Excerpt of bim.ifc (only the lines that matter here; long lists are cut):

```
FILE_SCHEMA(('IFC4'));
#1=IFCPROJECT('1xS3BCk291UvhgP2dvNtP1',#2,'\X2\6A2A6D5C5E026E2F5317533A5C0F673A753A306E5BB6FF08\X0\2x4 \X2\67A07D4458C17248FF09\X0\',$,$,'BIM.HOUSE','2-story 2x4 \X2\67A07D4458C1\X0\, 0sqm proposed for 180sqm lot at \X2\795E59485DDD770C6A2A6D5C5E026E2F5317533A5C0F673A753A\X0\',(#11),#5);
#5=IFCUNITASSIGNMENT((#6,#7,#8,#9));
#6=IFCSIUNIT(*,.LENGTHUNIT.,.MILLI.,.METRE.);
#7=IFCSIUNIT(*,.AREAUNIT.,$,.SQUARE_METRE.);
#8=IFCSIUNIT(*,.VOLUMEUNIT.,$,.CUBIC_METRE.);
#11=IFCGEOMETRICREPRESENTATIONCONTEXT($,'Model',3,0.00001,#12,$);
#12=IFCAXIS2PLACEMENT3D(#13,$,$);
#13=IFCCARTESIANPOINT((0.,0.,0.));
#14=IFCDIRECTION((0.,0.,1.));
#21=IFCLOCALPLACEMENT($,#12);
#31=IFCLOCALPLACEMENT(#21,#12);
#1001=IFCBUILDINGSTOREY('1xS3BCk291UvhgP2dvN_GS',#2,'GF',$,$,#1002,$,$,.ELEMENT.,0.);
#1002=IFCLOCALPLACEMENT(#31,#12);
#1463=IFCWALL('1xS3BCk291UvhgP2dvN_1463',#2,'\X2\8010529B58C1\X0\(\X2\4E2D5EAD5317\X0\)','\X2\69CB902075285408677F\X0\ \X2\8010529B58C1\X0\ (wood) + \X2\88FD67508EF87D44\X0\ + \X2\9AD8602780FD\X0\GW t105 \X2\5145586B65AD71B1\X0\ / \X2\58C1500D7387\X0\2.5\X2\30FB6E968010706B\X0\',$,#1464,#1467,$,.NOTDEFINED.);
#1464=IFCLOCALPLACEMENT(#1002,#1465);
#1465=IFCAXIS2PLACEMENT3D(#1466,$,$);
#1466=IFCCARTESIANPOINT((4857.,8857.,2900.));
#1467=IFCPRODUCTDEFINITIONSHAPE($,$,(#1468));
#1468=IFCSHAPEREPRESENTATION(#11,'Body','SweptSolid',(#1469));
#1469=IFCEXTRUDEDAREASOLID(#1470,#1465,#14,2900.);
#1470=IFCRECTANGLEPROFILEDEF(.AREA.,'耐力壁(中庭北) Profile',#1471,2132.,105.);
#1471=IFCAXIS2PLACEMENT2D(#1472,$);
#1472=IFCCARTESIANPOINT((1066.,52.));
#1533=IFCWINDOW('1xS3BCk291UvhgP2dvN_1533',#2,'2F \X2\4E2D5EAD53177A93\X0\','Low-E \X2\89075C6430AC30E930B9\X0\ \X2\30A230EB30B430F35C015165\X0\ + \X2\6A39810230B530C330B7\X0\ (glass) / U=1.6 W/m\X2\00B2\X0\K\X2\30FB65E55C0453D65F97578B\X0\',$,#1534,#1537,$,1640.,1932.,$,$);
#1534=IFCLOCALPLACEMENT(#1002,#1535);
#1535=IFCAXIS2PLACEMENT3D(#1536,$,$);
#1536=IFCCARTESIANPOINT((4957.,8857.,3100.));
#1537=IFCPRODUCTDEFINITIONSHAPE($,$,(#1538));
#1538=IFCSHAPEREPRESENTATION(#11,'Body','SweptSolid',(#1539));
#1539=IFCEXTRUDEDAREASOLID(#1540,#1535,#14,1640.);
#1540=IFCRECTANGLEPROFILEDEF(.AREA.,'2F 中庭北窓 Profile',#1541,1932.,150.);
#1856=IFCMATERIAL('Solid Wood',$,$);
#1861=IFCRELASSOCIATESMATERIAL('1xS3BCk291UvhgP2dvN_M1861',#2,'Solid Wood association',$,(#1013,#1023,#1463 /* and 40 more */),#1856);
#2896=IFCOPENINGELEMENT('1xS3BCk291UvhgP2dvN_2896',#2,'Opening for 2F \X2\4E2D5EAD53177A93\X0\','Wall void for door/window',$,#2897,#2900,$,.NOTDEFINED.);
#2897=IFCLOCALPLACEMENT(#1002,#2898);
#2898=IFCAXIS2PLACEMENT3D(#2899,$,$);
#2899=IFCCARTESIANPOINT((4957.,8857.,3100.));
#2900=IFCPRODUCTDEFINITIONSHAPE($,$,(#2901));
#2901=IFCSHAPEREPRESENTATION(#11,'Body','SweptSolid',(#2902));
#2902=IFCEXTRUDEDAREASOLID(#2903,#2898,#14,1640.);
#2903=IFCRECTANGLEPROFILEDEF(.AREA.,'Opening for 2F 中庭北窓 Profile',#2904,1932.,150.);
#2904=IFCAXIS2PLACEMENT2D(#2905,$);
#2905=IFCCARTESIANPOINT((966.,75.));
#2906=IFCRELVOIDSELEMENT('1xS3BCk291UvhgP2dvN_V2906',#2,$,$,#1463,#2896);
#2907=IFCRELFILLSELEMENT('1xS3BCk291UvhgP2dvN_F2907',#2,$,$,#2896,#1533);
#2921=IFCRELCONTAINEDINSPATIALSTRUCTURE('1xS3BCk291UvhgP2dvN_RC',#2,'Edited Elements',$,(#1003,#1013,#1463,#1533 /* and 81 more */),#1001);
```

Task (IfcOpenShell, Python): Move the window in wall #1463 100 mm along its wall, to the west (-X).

```python
import ifcopenshell
import ifcopenshell.api.geometry
import ifcopenshell.util.placement
import ifcopenshell.util.unit

model = ifcopenshell.open("bim.ifc")
unit_scale = ifcopenshell.util.unit.calculate_unit_scale(model)

window = model.by_guid("1xS3BCk291UvhgP2dvN_1533")
opening = window.FillsVoids[0].RelatingOpeningElement
wall = opening.VoidsElements[0].RelatingBuildingElement

wall_matrix = ifcopenshell.util.placement.get_local_placement(wall.ObjectPlacement)
shift = wall_matrix[:3, 0] * -0.1 / unit_scale
before = ifcopenshell.util.placement.get_local_placement(window.ObjectPlacement)[:3, 3].copy()

# The window is not placed relative to its opening, so move both.
for product in (opening, window):
    matrix = ifcopenshell.util.placement.get_local_placement(product.ObjectPlacement)
    matrix[:3, 3] += shift
    ifcopenshell.api.geometry.edit_object_placement(model, product=product, matrix=matrix, is_si=False)

after = ifcopenshell.util.placement.get_local_placement(window.ObjectPlacement)[:3, 3]
print("window moved by", (after - before).round(3) + 0.0)

model.write("bim_rev.ifc")
```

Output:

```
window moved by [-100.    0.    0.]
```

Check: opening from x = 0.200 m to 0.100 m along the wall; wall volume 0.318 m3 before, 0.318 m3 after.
